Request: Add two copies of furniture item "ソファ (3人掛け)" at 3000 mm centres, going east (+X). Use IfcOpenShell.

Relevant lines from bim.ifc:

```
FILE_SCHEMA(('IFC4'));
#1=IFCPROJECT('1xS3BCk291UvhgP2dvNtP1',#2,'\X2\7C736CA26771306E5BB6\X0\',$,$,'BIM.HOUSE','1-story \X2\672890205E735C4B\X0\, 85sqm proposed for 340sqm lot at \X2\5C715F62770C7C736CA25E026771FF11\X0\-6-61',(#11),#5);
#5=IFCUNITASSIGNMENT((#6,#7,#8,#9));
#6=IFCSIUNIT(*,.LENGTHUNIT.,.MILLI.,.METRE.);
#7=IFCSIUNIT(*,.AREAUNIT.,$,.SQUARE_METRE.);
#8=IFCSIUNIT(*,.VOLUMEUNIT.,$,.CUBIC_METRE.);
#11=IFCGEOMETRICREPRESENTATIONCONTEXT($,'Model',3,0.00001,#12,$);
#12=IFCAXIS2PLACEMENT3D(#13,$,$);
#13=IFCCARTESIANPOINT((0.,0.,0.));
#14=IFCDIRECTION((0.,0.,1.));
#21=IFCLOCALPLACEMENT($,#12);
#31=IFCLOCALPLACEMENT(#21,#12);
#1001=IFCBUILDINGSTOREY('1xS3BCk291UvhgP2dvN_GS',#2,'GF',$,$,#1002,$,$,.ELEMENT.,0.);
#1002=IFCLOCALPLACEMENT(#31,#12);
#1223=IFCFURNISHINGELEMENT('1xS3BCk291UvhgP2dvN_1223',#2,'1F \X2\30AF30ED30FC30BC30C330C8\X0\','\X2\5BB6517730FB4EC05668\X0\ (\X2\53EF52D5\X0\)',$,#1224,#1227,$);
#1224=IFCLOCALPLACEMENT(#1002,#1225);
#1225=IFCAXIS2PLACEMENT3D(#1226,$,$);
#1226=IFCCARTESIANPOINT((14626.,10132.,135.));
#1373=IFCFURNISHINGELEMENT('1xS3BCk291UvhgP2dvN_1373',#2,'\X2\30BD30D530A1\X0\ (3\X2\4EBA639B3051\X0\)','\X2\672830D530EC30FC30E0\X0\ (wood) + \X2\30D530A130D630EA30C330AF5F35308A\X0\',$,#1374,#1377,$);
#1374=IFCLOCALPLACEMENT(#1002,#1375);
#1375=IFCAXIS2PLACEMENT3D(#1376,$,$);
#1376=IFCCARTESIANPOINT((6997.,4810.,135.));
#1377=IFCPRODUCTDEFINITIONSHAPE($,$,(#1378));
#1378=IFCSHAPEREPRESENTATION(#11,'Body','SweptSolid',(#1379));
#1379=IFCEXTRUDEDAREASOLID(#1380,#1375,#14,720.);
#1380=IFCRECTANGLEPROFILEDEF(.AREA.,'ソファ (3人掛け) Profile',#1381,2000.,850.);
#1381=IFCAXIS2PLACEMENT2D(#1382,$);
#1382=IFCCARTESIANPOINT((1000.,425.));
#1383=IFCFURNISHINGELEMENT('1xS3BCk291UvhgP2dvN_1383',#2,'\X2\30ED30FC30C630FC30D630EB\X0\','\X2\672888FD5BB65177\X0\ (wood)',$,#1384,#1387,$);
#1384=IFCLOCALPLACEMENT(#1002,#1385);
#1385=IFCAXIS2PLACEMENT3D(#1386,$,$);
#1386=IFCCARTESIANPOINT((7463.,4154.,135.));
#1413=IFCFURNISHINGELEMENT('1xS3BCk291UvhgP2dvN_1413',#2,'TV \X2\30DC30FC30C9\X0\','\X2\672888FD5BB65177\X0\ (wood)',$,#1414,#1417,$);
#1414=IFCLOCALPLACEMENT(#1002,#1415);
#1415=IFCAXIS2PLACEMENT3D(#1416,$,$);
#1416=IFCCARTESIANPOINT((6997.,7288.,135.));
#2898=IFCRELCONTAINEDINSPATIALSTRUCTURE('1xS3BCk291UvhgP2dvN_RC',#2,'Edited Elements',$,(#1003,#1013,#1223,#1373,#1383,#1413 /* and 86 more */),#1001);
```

```python
import numpy as np
import ifcopenshell
import ifcopenshell.api.geometry
import ifcopenshell.api.root
import ifcopenshell.util.element
import ifcopenshell.util.placement
import ifcopenshell.util.unit

model = ifcopenshell.open("bim.ifc")
unit_scale = ifcopenshell.util.unit.calculate_unit_scale(model)


def reuse_history(source, copy):
    """copy_class also copies each property set's owner history, people and application; keep the originals."""
    for rel in copy.IsDefinedBy:
        if rel.is_a("IfcRelDefinesByProperties") and (history := rel.RelatingPropertyDefinition.OwnerHistory):
            rel.RelatingPropertyDefinition.OwnerHistory = source.OwnerHistory
            ifcopenshell.util.element.remove_deep2(model, history)


source = model.by_id(1373)
base = ifcopenshell.util.placement.get_local_placement(source.ObjectPlacement)
step = np.array([1.0, 0.0, 0.0]) * 3 / unit_scale

for i in range(1, 3):
    copy = ifcopenshell.api.root.copy_class(model, product=source)
    copy.Representation = ifcopenshell.util.element.copy_deep(
        model, source.Representation, exclude=["IfcGeometricRepresentationContext", "IfcRepresentationMap"]
    )
    reuse_history(source, copy)
    matrix = base.copy()
    matrix[:3, 3] += i * step
    print("added at", matrix[:3, 3].round(3) + 0.0)
    ifcopenshell.api.geometry.edit_object_placement(model, product=copy, matrix=matrix, is_si=False)

model.write("bim_rev.ifc")
```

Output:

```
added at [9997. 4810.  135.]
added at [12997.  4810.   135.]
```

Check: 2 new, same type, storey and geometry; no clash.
